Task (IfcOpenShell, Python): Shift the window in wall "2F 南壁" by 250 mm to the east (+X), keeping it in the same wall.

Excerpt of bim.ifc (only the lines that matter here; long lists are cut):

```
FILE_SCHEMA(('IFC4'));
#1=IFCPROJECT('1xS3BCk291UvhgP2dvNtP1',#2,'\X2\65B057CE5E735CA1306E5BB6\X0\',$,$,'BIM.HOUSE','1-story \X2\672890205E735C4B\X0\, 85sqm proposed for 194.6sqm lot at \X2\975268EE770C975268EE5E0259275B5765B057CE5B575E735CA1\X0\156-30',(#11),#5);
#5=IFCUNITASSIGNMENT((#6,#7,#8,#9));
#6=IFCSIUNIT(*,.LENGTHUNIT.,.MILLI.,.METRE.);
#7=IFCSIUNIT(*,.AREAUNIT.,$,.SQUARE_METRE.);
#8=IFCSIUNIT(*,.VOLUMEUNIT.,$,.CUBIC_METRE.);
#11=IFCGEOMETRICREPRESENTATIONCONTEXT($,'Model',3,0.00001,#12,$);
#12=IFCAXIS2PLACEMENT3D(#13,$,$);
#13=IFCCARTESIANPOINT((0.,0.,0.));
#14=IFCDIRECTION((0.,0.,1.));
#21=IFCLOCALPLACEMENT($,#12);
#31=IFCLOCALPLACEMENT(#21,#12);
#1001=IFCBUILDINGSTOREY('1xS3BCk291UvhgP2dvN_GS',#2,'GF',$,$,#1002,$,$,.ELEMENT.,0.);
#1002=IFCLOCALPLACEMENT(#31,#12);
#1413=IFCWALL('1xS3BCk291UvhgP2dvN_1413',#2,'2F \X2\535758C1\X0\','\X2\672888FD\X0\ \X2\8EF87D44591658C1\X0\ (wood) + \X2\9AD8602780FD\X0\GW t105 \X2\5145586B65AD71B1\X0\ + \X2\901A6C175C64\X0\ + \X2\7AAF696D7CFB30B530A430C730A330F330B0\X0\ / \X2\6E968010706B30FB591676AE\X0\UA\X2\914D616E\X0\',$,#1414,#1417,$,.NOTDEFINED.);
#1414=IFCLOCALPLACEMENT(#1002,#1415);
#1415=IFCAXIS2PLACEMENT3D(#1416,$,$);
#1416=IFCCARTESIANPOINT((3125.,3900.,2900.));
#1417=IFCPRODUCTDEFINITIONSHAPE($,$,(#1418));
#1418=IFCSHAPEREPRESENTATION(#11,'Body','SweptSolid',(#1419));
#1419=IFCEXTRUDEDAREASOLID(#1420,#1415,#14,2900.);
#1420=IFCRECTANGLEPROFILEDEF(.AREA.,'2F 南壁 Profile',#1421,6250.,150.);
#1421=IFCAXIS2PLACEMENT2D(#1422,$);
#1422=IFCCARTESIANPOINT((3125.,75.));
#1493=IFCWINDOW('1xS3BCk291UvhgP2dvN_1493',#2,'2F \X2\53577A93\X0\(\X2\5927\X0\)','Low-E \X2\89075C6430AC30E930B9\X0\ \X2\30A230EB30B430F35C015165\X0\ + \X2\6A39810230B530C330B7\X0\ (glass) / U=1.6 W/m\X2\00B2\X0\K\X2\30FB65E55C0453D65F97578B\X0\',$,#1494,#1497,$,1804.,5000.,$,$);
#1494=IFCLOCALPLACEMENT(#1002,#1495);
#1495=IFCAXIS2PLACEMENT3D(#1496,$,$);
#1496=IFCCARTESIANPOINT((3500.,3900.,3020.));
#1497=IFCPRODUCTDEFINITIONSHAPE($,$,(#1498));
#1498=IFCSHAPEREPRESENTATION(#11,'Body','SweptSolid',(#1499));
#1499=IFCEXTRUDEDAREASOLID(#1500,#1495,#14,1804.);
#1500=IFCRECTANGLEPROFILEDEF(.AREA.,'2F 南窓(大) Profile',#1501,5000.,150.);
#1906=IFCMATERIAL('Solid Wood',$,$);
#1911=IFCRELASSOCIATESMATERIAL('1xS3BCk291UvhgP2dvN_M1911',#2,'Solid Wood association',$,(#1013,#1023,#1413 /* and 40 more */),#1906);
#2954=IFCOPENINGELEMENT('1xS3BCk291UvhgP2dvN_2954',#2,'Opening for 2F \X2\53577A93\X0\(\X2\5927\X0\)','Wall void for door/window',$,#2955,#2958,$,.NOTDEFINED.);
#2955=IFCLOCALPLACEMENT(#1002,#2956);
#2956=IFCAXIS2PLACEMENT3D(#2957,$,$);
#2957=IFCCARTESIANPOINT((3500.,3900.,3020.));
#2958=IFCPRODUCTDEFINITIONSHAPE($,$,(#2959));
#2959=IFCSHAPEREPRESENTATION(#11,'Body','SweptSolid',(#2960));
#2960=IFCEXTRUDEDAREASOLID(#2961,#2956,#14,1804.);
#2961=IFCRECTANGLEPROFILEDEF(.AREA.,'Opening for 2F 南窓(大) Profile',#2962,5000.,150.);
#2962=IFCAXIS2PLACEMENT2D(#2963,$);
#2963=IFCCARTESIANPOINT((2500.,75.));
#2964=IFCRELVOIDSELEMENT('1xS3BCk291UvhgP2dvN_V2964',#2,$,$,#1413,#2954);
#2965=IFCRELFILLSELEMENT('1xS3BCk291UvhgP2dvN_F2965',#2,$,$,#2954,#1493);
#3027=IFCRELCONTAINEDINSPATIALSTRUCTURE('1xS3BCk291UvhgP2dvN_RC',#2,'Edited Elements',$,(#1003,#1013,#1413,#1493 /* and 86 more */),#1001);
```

```python
import ifcopenshell
import ifcopenshell.api.geometry
import ifcopenshell.util.placement

model = ifcopenshell.open("bim.ifc")

window = model.by_guid("1xS3BCk291UvhgP2dvN_1493")
opening = window.FillsVoids[0].RelatingOpeningElement
wall = opening.VoidsElements[0].RelatingBuildingElement

wall_matrix = ifcopenshell.util.placement.get_local_placement(wall.ObjectPlacement)
shift = wall_matrix[:3, 0] * 250.0
before = ifcopenshell.util.placement.get_local_placement(window.ObjectPlacement)[:3, 3].copy()

# The window is not placed relative to its opening, so move both.
for product in (opening, window):
    matrix = ifcopenshell.util.placement.get_local_placement(product.ObjectPlacement)
    matrix[:3, 3] += shift
    ifcopenshell.api.geometry.edit_object_placement(model, product=product, matrix=matrix, is_si=False)

after = ifcopenshell.util.placement.get_local_placement(window.ObjectPlacement)[:3, 3]
print("window moved by", (after - before).round(3) + 0.0)

model.write("bim-out.ifc")
```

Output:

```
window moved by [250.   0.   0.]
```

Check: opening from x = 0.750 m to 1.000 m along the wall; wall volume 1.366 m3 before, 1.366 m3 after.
